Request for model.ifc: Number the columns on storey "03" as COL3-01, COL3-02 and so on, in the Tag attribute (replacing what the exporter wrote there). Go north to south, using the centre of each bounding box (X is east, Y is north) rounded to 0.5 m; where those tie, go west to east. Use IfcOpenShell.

First a look at what the model holds.

```python
import ifcopenshell
import ifcopenshell.util.element
import ifcopenshell.util.placement

model = ifcopenshell.open("model.ifc")
print(model.schema)
storey = next(s for s in model.by_type("IfcBuildingStorey") if s.Name == "03")
columns = [e for e in ifcopenshell.util.element.get_decomposition(storey) if e.is_a("IfcColumn")]
for e in sorted(columns, key=lambda e: e.id()):
    origin = ifcopenshell.util.placement.get_local_placement(e.ObjectPlacement)[:3, 3]
    print(e.id(), e.Tag, e.Name, origin.round(2) + 0.0, sep=" | ")
```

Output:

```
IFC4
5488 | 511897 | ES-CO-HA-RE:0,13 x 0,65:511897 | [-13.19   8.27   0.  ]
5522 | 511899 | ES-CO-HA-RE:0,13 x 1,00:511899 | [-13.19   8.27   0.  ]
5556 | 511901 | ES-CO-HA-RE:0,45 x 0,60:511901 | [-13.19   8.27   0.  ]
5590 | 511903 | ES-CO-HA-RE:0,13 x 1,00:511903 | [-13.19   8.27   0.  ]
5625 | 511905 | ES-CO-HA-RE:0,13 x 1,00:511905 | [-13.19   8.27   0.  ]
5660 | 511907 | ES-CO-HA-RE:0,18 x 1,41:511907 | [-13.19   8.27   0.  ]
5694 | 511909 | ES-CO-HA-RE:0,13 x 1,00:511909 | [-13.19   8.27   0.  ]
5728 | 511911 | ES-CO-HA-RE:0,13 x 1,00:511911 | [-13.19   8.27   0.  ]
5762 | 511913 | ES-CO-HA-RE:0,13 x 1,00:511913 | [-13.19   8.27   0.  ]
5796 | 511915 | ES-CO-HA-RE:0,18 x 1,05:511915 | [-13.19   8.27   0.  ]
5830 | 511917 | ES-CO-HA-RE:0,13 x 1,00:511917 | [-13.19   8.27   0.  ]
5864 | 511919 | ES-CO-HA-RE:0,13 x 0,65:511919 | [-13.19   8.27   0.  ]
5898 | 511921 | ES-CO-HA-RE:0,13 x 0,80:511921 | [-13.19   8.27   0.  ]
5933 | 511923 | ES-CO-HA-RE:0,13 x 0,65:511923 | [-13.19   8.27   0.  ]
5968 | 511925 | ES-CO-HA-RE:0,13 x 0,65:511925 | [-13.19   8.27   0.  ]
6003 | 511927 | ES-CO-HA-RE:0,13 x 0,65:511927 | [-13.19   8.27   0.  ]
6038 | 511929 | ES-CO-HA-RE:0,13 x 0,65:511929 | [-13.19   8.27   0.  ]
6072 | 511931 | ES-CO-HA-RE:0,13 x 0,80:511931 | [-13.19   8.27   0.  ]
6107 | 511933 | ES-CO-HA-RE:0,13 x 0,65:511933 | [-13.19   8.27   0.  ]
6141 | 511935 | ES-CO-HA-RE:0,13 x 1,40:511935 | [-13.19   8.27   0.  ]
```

```python
import ifcopenshell
import ifcopenshell.geom
import ifcopenshell.util.element
import ifcopenshell.util.shape

model = ifcopenshell.open("model.ifc")
settings = ifcopenshell.geom.settings()
settings.set("use-world-coords", True)


def centre(element):
    shape = ifcopenshell.geom.create_shape(settings, element)
    return ifcopenshell.util.shape.get_bbox_centroid(shape.geometry)


storey = next(s for s in model.by_type("IfcBuildingStorey") if s.Name == "03")
columns = [e for e in ifcopenshell.util.element.get_decomposition(storey) if e.is_a("IfcColumn")]

# Insertion points can sit at a corner or the storey origin, so sort by the geometry (in metres).
centres = {e: centre(e) for e in columns}
columns.sort(key=lambda e: (-round(centres[e][1] / 0.5), centres[e][0]))

for i, e in enumerate(columns, start=1):
    number = f"COL3-{i:02d}"
    e.Tag = number
    print(e.id(), number)

model.write("model_updated.ifc")
```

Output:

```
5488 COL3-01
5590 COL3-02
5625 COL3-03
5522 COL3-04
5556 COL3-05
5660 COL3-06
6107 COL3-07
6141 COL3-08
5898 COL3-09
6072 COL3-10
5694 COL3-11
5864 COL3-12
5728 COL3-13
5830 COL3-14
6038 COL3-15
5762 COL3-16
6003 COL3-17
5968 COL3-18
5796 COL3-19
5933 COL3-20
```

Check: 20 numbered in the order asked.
